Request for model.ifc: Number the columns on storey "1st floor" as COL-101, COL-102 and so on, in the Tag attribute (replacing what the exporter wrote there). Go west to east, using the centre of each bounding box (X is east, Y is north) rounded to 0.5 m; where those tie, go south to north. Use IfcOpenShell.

First a look at what the model holds.

```python
import ifcopenshell
import ifcopenshell.util.element
import ifcopenshell.util.placement

model = ifcopenshell.open("model.ifc")
print(model.schema)
storey = next(s for s in model.by_type("IfcBuildingStorey") if s.Name == "1st floor")
columns = [e for e in ifcopenshell.util.element.get_decomposition(storey) if e.is_a("IfcColumn")]
for e in sorted(columns, key=lambda e: e.id()):
    origin = ifcopenshell.util.placement.get_local_placement(e.ObjectPlacement)[:3, 3]
    print(e.id(), e.Tag, e.Name, origin.round(2) + 0.0, sep=" | ")
```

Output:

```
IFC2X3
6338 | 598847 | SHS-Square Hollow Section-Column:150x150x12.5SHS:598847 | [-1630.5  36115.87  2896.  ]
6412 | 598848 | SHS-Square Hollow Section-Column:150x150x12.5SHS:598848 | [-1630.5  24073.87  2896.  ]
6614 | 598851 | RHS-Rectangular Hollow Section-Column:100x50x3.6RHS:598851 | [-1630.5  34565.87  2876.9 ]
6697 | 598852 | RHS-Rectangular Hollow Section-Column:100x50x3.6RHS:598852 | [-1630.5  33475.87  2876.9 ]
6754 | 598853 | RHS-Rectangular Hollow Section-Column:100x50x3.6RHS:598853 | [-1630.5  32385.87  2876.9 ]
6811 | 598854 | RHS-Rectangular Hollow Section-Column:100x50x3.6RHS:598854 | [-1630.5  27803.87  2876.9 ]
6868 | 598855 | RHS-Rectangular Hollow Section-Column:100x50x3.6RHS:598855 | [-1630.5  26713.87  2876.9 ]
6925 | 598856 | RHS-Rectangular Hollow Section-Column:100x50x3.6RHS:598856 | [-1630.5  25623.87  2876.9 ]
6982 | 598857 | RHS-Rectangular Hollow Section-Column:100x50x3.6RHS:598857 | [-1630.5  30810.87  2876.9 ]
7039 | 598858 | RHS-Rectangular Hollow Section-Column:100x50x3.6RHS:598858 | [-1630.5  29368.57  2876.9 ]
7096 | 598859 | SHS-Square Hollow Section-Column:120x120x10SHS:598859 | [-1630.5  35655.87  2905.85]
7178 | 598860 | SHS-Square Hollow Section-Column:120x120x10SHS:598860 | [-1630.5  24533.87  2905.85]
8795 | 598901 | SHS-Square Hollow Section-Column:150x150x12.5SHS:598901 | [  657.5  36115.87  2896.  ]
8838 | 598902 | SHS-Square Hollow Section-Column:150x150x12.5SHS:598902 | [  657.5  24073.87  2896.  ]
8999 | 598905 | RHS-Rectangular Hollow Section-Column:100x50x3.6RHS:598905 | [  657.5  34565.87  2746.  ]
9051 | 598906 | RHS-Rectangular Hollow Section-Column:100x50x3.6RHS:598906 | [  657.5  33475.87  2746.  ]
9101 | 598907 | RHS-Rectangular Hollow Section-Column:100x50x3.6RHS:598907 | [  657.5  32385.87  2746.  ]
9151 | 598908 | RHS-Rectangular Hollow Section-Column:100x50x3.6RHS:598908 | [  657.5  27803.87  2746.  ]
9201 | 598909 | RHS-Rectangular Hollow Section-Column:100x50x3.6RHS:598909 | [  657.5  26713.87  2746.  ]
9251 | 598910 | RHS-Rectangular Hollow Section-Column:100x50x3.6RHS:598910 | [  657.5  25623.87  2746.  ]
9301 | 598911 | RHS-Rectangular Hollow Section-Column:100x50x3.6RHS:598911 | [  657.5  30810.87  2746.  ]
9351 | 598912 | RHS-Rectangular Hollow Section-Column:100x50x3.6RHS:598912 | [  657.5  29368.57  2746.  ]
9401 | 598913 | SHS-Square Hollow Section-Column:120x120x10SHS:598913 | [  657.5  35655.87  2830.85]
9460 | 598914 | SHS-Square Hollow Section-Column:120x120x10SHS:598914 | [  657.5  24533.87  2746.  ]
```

```python
import ifcopenshell
import ifcopenshell.geom
import ifcopenshell.util.element
import ifcopenshell.util.shape

model = ifcopenshell.open("model.ifc")
settings = ifcopenshell.geom.settings()
settings.set("use-world-coords", True)


def centre(element):
    shape = ifcopenshell.geom.create_shape(settings, element)
    return ifcopenshell.util.shape.get_bbox_centroid(shape.geometry)


storey = next(s for s in model.by_type("IfcBuildingStorey") if s.Name == "1st floor")
columns = [e for e in ifcopenshell.util.element.get_decomposition(storey) if e.is_a("IfcColumn")]

# Insertion points can sit at a corner or the storey origin, so sort by the geometry (in metres).
centres = {e: centre(e) for e in columns}
columns.sort(key=lambda e: (round(centres[e][0] / 0.5), centres[e][1]))

for i, e in enumerate(columns, start=1):
    number = f"COL-1{i:02d}"
    e.Tag = number
    print(e.id(), number)

model.write("model_edited.ifc")
```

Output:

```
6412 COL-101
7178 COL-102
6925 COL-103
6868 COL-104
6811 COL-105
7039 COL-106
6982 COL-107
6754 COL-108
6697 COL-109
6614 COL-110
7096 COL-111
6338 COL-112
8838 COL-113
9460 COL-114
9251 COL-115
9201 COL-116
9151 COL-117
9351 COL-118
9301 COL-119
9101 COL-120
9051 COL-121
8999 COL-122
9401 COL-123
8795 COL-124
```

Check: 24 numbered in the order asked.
